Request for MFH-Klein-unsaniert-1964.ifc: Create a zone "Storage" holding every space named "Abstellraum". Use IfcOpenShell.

First a look at what the model holds.

```python
import ifcopenshell

model = ifcopenshell.open("MFH-Klein-unsaniert-1964.ifc")
print(model.schema)
seen = {}
for space in model.by_type("IfcSpace"):
    seen[space.Name] = seen.get(space.Name, 0) + 1
for name, count in sorted(seen.items(), key=str):
    print(count, "x", name)
print("zones:", [z.Name for z in model.by_type("IfcZone")][:20])
```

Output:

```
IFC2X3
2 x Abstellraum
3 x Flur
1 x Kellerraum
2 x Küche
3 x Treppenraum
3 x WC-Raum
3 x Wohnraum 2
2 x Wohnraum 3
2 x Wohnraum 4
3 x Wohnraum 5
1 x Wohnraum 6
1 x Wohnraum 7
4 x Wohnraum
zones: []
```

```python
import ifcopenshell
import ifcopenshell.api.group
import ifcopenshell.api.root

model = ifcopenshell.open("MFH-Klein-unsaniert-1964.ifc")

names = {"Abstellraum"}
spaces = [s for s in model.by_type("IfcSpace") if s.Name in names]

zone = ifcopenshell.api.root.create_entity(model, ifc_class="IfcZone", name="Storage")
ifcopenshell.api.group.assign_group(model, products=spaces, group=zone)
print(len(spaces), "spaces in", zone.Name)

model.write("MFH-Klein-unsaniert-1964-out.ifc")
```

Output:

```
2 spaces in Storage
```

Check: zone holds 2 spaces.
